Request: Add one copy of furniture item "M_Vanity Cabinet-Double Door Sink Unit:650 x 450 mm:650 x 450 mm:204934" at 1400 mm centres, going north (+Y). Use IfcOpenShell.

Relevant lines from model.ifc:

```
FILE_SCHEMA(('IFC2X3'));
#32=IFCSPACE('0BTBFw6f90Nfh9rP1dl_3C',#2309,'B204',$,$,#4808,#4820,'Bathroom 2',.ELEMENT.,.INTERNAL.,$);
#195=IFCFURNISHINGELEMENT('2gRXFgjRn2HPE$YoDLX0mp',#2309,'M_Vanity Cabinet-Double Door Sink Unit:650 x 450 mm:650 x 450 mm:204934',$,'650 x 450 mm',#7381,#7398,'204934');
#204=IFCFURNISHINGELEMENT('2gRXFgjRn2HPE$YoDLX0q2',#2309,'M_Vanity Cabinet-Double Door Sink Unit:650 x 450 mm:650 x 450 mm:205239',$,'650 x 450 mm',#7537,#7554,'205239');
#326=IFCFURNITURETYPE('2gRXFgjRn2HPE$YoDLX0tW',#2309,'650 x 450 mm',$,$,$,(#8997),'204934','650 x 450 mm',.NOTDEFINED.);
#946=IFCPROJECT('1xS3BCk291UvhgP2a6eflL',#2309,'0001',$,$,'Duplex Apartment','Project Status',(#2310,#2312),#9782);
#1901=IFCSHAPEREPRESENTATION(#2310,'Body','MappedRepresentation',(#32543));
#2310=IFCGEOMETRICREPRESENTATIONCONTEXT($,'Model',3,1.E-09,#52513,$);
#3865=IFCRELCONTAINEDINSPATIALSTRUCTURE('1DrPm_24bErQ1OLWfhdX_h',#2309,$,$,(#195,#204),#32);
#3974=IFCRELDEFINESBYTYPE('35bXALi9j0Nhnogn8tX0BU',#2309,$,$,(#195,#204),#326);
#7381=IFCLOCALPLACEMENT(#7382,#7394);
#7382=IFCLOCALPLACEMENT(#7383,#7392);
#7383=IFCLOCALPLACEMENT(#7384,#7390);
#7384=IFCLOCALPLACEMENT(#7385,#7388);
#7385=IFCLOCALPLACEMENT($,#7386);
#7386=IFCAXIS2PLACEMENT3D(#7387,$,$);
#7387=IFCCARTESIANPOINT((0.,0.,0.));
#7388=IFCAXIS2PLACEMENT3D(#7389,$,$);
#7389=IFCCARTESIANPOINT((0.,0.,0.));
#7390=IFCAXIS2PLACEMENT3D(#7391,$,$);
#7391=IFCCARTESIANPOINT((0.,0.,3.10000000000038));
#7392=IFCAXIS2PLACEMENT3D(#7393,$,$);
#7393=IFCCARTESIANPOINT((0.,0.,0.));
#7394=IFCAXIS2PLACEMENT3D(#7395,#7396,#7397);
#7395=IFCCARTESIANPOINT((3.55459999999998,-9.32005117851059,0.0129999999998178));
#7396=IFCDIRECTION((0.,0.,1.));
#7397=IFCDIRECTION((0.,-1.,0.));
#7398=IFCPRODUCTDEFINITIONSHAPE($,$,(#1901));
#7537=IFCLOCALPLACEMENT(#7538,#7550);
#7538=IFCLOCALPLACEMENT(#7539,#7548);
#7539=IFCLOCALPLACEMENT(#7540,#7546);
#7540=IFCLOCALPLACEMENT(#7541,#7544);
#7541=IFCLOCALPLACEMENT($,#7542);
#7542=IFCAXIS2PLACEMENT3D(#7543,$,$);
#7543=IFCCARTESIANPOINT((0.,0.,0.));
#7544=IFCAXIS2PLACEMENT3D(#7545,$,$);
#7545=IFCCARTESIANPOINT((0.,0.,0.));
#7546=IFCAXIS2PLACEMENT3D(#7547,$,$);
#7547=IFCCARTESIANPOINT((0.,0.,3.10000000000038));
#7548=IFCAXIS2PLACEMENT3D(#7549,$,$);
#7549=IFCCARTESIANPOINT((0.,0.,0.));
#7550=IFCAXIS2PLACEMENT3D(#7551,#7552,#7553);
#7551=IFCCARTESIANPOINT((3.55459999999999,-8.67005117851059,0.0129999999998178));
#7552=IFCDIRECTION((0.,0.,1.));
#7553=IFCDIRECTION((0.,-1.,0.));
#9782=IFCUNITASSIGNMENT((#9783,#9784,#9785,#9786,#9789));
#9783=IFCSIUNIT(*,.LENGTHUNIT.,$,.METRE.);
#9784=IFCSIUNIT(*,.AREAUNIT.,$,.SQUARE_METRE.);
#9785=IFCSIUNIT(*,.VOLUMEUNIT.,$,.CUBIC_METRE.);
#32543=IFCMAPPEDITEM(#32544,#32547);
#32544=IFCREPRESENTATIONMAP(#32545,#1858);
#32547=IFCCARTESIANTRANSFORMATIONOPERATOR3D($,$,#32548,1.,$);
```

```python
import numpy as np
import ifcopenshell
import ifcopenshell.api.geometry
import ifcopenshell.api.root
import ifcopenshell.util.element
import ifcopenshell.util.placement
import ifcopenshell.util.unit

model = ifcopenshell.open("model.ifc")
unit_scale = ifcopenshell.util.unit.calculate_unit_scale(model)


def reuse_history(source, copy):
    """copy_class also copies each property set's owner history, people and application; keep the originals."""
    for rel in copy.IsDefinedBy:
        if rel.is_a("IfcRelDefinesByProperties") and (history := rel.RelatingPropertyDefinition.OwnerHistory):
            rel.RelatingPropertyDefinition.OwnerHistory = source.OwnerHistory
            ifcopenshell.util.element.remove_deep2(model, history)


source = model.by_guid("2gRXFgjRn2HPE$YoDLX0mp")
base = ifcopenshell.util.placement.get_local_placement(source.ObjectPlacement)
step = np.array([0.0, 1.0, 0.0]) * 1.4 / unit_scale

for i in range(1, 2):
    copy = ifcopenshell.api.root.copy_class(model, product=source)
    copy.Representation = ifcopenshell.util.element.copy_deep(
        model, source.Representation, exclude=["IfcGeometricRepresentationContext", "IfcRepresentationMap"]
    )
    copy.Name = "M_Vanity Cabinet-Double Door Sink Unit:650 x 450 mm:650 x 450 mm"
    copy.Tag = None
    reuse_history(source, copy)
    matrix = base.copy()
    matrix[:3, 3] += i * step
    print("added at", matrix[:3, 3].round(3) + 0.0)
    ifcopenshell.api.geometry.edit_object_placement(model, product=copy, matrix=matrix, is_si=False)

model.write("model_edited.ifc")
```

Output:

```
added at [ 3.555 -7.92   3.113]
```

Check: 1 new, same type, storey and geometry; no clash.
